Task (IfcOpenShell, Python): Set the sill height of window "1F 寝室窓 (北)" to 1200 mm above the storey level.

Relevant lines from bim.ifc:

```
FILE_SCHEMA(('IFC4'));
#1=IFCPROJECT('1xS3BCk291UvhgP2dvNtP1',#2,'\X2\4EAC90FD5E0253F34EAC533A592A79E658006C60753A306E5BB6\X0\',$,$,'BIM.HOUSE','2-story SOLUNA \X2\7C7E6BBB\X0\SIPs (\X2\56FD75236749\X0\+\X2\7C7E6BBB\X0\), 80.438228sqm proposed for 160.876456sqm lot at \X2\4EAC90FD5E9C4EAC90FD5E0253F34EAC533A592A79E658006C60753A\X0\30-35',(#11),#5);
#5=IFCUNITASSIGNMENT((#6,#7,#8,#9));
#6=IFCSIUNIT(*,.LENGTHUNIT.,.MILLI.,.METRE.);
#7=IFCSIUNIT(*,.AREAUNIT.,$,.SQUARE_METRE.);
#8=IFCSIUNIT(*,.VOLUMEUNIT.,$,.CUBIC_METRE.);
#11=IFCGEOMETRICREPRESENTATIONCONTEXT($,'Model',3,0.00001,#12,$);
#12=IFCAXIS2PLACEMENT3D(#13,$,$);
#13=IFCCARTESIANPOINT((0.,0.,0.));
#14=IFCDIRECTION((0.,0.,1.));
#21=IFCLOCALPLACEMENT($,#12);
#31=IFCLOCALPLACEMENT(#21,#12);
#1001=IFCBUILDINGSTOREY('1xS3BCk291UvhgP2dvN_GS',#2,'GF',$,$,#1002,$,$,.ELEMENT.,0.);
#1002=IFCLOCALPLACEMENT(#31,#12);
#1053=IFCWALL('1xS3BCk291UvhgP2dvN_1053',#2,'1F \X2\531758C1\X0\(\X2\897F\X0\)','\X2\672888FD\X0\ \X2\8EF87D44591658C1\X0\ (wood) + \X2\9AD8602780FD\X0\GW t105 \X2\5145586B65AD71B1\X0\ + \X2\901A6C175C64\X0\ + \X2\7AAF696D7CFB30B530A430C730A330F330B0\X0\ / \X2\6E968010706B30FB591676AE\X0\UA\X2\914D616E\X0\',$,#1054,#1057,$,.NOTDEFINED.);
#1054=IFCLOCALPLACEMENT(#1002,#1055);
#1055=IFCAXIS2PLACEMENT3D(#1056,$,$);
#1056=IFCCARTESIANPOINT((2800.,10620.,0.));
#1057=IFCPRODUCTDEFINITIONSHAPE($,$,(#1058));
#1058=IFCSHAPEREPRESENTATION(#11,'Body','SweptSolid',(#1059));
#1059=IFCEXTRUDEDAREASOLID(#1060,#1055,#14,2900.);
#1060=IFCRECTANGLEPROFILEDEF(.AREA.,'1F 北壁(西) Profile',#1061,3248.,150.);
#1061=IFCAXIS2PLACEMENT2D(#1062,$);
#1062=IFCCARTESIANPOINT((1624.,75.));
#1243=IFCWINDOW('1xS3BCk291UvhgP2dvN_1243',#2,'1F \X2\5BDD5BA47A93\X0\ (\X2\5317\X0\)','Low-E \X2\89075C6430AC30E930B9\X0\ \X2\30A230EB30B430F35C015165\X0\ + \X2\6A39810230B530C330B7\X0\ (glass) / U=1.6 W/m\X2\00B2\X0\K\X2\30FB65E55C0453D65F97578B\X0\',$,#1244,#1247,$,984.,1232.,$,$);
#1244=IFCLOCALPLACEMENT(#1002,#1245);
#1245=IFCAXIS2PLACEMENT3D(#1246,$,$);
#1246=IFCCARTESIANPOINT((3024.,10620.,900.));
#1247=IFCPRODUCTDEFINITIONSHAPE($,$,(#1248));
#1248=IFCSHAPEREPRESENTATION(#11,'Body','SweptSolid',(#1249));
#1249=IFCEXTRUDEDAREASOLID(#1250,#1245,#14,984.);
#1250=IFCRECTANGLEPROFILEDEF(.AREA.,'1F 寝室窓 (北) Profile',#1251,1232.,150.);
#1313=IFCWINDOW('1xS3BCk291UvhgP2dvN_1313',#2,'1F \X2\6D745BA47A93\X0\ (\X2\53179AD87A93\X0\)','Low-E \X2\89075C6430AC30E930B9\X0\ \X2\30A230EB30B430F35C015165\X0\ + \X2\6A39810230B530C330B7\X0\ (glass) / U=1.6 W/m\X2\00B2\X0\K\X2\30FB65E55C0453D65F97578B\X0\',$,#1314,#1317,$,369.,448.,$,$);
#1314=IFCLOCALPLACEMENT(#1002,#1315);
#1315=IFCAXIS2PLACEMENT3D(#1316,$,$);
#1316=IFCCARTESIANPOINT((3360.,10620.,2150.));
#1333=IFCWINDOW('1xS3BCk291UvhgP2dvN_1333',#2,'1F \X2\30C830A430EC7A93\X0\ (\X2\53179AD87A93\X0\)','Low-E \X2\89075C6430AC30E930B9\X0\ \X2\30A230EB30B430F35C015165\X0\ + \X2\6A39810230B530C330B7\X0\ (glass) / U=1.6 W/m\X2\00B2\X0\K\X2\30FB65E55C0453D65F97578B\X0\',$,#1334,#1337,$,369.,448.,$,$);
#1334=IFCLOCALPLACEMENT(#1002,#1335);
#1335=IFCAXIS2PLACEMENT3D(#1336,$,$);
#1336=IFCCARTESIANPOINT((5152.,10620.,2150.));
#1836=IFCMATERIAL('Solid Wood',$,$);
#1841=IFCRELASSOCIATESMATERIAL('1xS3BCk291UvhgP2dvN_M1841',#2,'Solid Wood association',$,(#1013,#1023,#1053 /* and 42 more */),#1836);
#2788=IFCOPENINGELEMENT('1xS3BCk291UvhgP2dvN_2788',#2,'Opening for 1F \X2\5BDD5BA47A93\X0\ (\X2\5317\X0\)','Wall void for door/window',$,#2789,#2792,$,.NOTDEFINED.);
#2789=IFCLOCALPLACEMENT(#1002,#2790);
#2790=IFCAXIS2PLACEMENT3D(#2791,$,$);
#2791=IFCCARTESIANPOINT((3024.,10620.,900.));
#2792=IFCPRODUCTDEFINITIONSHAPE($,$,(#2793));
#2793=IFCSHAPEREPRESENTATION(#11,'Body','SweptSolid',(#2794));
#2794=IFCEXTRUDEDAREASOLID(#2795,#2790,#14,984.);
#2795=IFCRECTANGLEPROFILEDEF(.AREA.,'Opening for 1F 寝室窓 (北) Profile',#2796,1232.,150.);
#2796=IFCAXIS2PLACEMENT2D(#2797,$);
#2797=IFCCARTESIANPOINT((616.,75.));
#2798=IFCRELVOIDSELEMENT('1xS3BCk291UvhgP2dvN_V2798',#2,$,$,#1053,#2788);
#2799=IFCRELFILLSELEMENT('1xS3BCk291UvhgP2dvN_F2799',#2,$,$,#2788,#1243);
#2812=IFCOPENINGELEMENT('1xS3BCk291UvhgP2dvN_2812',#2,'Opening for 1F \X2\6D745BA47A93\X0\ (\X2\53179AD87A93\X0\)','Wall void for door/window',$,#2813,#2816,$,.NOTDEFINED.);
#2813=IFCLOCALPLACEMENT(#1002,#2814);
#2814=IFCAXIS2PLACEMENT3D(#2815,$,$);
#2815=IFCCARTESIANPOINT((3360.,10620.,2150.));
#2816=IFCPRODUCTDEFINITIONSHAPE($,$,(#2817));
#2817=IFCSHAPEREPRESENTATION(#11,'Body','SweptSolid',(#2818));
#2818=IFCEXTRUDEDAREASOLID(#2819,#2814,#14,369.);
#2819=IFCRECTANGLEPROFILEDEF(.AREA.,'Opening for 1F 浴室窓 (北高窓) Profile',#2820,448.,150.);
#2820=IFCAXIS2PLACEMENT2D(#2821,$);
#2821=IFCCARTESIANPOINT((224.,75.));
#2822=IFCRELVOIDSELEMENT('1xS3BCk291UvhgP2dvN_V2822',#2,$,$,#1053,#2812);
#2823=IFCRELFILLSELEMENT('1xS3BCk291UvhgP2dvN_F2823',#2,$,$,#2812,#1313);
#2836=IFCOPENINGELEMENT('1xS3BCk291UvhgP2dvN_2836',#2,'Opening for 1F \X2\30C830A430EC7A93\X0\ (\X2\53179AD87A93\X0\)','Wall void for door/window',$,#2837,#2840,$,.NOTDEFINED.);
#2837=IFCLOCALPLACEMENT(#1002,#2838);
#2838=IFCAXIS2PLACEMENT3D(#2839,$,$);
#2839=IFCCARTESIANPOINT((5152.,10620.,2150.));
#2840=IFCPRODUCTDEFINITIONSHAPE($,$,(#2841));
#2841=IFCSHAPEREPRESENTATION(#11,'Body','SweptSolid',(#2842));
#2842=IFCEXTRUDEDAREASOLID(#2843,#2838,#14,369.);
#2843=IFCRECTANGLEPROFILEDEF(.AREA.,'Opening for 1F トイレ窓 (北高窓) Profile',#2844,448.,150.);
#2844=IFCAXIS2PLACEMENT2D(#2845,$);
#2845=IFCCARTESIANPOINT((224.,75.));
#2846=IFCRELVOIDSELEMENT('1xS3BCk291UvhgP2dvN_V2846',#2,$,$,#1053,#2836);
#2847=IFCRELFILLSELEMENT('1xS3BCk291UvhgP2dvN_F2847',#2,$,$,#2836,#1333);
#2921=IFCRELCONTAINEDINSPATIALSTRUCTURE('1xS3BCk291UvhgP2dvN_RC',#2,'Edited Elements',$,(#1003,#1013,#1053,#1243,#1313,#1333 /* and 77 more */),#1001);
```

```python
import numpy as np
import ifcopenshell
import ifcopenshell.api.geometry
import ifcopenshell.geom
import ifcopenshell.util.element
import ifcopenshell.util.placement
import ifcopenshell.util.shape
import ifcopenshell.util.unit

model = ifcopenshell.open("bim.ifc")
unit_scale = ifcopenshell.util.unit.calculate_unit_scale(model)

window = model.by_guid("1xS3BCk291UvhgP2dvN_1243")
opening = window.FillsVoids[0].RelatingOpeningElement
storey = ifcopenshell.util.element.get_container(window, ifc_class="IfcBuildingStorey")
level = ifcopenshell.util.placement.get_local_placement(storey.ObjectPlacement)[2, 3]

# The opening's origin need not be at the sill, so measure its lowest point.
shape = ifcopenshell.geom.create_shape(ifcopenshell.geom.settings(), opening)
bottom = ifcopenshell.util.shape.get_shape_bottom_elevation(shape, shape.geometry) / unit_scale
dz = level + 1200.0 - bottom

shift = np.array([0.0, 0.0, dz])
# The window is not placed relative to its opening, so move both.
for product in (opening, window):
    matrix = ifcopenshell.util.placement.get_local_placement(product.ObjectPlacement)
    matrix[:3, 3] += shift
    ifcopenshell.api.geometry.edit_object_placement(model, product=product, matrix=matrix, is_si=False)

print(f"moved by {dz * unit_scale:+.3f} m")

model.write("bim_edited.ifc")
```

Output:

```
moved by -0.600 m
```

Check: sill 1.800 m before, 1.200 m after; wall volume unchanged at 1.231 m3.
